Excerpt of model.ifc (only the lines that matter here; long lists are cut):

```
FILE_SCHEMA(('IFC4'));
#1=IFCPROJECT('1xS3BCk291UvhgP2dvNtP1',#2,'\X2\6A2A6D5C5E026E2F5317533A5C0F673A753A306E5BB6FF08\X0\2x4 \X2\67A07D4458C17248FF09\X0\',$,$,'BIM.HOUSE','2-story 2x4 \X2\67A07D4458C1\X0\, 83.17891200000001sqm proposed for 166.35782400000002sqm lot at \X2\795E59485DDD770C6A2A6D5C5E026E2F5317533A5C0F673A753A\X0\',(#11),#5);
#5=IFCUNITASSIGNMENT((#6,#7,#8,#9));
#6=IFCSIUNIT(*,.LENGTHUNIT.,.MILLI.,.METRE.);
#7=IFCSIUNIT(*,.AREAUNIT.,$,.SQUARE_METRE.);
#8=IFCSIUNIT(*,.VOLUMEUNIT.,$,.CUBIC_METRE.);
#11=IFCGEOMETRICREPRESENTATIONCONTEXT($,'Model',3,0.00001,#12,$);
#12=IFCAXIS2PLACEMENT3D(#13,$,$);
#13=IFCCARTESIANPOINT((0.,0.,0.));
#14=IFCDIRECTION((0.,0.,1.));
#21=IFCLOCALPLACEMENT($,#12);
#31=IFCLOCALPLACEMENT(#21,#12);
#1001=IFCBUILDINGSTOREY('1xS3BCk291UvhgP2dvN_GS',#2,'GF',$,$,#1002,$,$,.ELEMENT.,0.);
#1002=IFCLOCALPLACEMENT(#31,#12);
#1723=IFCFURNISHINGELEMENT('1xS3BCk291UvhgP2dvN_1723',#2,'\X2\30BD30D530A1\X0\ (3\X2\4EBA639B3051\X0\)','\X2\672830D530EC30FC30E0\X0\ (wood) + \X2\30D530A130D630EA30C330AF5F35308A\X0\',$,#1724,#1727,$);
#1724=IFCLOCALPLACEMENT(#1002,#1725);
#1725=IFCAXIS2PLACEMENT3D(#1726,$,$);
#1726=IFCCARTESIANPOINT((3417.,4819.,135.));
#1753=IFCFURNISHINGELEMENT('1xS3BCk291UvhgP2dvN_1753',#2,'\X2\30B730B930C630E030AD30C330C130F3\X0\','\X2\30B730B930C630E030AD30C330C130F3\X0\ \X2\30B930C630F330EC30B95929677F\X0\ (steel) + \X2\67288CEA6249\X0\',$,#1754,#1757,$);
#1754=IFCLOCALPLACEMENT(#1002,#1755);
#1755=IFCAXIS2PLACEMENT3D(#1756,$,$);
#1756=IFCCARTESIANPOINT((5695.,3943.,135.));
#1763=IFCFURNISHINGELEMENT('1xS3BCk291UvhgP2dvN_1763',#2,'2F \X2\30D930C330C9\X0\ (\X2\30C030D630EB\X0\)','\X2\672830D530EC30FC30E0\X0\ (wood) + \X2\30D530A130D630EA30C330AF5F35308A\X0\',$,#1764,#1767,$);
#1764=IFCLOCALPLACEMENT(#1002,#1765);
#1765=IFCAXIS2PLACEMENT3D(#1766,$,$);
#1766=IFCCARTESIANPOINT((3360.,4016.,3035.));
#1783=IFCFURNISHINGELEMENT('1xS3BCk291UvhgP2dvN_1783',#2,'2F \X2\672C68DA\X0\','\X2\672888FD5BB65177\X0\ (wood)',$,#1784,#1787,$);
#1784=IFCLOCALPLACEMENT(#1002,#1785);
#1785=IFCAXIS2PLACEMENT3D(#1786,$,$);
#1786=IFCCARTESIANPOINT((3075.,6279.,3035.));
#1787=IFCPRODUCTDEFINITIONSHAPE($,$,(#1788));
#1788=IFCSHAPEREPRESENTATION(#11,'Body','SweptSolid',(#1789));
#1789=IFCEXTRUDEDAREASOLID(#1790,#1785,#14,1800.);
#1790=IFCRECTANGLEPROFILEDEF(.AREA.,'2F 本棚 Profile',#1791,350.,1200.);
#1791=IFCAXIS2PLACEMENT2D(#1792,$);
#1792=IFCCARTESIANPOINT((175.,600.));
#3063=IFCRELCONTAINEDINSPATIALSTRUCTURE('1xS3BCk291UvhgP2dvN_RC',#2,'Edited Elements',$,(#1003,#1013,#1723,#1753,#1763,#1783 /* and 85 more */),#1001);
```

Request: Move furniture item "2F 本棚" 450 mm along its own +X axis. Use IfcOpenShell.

```python
import ifcopenshell
import ifcopenshell.api.geometry
import ifcopenshell.util.placement
import ifcopenshell.util.unit

model = ifcopenshell.open("model.ifc")
unit_scale = ifcopenshell.util.unit.calculate_unit_scale(model)

item = model.by_guid("1xS3BCk291UvhgP2dvN_1783")
matrix = ifcopenshell.util.placement.get_local_placement(item.ObjectPlacement)
matrix[:3, 3] += matrix[:3, 0] * 0.45 / unit_scale
ifcopenshell.api.geometry.edit_object_placement(model, product=item, matrix=matrix, is_si=False)

print(ifcopenshell.util.placement.get_local_placement(item.ObjectPlacement).round(3) + 0.0)

model.write("model_v2.ifc")
```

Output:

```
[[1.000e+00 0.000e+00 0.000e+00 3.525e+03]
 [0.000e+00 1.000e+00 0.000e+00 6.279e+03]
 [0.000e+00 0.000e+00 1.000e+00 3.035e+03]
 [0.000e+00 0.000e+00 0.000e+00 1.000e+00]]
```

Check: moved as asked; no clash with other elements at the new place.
